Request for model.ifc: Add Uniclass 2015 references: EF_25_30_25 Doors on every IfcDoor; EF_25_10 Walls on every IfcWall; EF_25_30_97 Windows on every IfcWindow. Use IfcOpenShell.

First a look at what the model holds.

```python
import ifcopenshell

model = ifcopenshell.open("model.ifc")
print(model.schema)
print("classifications:", [c.Name for c in model.by_type("IfcClassification")])
for ifc_class in ("IfcDoor", "IfcRoof", "IfcStair", "IfcWall", "IfcWindow"):
    print(ifc_class, len(model.by_type(ifc_class)))
```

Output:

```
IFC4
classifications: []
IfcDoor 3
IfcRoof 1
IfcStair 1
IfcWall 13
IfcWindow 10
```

```python
import ifcopenshell
import ifcopenshell.api.classification

model = ifcopenshell.open("model.ifc")

system = ifcopenshell.api.classification.add_classification(model, classification="Uniclass 2015")

codes = {
    "IfcDoor": ("EF_25_30_25", "Doors"),
    "IfcWall": ("EF_25_10", "Walls"),
    "IfcWindow": ("EF_25_30_97", "Windows"),
}
for ifc_class, (code, name) in codes.items():
    products = model.by_type(ifc_class)
    ifcopenshell.api.classification.add_reference(
        model, products=products, classification=system, identification=code, name=name
    )
    print(code, len(products))

model.write("model_v2.ifc")
```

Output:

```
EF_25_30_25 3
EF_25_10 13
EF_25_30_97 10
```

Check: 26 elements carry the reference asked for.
